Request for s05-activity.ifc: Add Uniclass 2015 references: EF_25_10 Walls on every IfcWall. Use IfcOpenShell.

First a look at what the model holds.

```python
import ifcopenshell

model = ifcopenshell.open("s05-activity.ifc")
print(model.schema)
print("classifications:", [c.Name for c in model.by_type("IfcClassification")])
for ifc_class in ("IfcDoor", "IfcRoof", "IfcStair", "IfcWall", "IfcWindow"):
    print(ifc_class, len(model.by_type(ifc_class)))
```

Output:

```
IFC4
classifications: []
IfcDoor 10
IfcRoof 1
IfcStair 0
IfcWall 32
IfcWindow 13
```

```python
import ifcopenshell
import ifcopenshell.api.classification

model = ifcopenshell.open("s05-activity.ifc")

system = ifcopenshell.api.classification.add_classification(model, classification="Uniclass 2015")

codes = {
    "IfcWall": ("EF_25_10", "Walls"),
}
for ifc_class, (code, name) in codes.items():
    products = model.by_type(ifc_class)
    ifcopenshell.api.classification.add_reference(
        model, products=products, classification=system, identification=code, name=name
    )
    print(code, len(products))

model.write("s05-activity_edited.ifc")
```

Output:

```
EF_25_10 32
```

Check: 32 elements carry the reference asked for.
